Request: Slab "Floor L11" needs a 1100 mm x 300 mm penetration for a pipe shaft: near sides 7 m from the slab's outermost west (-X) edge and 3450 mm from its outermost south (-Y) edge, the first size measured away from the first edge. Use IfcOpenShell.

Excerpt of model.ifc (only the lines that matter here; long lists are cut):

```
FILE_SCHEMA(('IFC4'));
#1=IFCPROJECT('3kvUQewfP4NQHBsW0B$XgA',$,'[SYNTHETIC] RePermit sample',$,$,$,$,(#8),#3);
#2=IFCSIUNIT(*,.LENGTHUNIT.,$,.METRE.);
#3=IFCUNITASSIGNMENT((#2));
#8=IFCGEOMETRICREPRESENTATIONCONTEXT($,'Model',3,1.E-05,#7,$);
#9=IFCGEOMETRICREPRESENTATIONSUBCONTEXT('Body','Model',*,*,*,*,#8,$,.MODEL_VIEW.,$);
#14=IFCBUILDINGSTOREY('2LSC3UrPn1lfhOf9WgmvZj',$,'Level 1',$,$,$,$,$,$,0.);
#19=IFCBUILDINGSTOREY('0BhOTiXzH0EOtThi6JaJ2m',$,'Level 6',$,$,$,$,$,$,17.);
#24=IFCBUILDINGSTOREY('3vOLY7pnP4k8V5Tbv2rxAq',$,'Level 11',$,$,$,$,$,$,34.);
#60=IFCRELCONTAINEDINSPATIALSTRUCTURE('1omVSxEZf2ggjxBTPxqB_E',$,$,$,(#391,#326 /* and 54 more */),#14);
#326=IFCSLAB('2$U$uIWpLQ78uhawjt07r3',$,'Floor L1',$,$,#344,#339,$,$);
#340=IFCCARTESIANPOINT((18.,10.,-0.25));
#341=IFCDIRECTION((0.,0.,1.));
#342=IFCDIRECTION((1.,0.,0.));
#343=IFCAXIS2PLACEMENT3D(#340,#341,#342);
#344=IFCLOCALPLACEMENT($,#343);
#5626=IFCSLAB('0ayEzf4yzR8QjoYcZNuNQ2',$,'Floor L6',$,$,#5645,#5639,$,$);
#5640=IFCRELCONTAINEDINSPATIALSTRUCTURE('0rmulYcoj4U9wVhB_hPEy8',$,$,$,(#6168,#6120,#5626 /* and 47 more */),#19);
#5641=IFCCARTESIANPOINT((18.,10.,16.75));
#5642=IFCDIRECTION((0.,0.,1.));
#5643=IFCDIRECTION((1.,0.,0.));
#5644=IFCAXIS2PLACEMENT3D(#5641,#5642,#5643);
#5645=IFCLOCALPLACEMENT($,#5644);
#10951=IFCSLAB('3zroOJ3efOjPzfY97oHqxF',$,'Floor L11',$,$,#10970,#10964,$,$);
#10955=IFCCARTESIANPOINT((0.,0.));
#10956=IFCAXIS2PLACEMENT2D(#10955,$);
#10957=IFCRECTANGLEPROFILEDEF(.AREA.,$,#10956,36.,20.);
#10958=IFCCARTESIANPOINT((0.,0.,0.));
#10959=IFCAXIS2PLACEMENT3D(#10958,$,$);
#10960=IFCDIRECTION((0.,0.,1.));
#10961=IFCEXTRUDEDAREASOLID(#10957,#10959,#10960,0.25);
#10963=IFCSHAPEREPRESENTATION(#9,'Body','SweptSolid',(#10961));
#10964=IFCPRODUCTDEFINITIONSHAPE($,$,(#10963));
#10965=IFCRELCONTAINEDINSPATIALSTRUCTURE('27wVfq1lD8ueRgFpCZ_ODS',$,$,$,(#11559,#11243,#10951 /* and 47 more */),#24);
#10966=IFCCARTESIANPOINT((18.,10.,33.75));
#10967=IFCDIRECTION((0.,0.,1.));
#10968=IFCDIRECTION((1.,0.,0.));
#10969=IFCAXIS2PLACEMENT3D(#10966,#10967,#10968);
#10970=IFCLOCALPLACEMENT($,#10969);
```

```python
import numpy as np
import ifcopenshell
import ifcopenshell.api.feature
import ifcopenshell.api.geometry
import ifcopenshell.api.root
import ifcopenshell.geom
import ifcopenshell.util.placement
import ifcopenshell.util.representation
import ifcopenshell.util.shape
import ifcopenshell.util.unit

model = ifcopenshell.open("model.ifc")
unit_scale = ifcopenshell.util.unit.calculate_unit_scale(model)
settings = ifcopenshell.geom.settings()


def volume(element):
    """Net volume in cubic metres, openings subtracted."""
    shape = ifcopenshell.geom.create_shape(settings, element)
    return ifcopenshell.util.shape.get_volume(shape.geometry)


slab = model.by_guid("3zroOJ3efOjPzfY97oHqxF")
before = volume(slab)

# Extent in the slab's own axes, in metres. The edges named are its -X and -Y sides.
slab_shape = ifcopenshell.geom.create_shape(settings, slab)
vertices = ifcopenshell.util.shape.get_vertices(slab_shape.geometry)
x_min, y_min, bottom = vertices.min(axis=0)
top = vertices[:, 2].max()

opening = ifcopenshell.api.root.create_entity(model, ifc_class="IfcOpeningElement", name="Pipe shaft opening", predefined_type="OPENING")
context = ifcopenshell.util.representation.get_context(model, "Model", "Body", "MODEL_VIEW")
width, depth = 1.1, 0.3
outline = [(0.0, 0.0), (width, 0.0), (width, depth), (0.0, depth), (0.0, 0.0)]
# Overshoot both faces by 50 mm so the cut is clean.
shape = ifcopenshell.api.geometry.add_slab_representation(
    model, context=context, depth=top - bottom + 0.1, polyline=outline
)
ifcopenshell.api.geometry.assign_representation(model, product=opening, representation=shape)

matrix = ifcopenshell.util.placement.get_local_placement(slab.ObjectPlacement)
matrix[:, 3] = matrix @ np.append(np.array([x_min + 7, y_min + 3.45, bottom - 0.05]) / unit_scale, 1.0)
ifcopenshell.api.geometry.edit_object_placement(model, product=opening, matrix=matrix, is_si=False)
ifcopenshell.api.feature.add_feature(model, feature=opening, element=slab)

after = volume(slab)

print(f"slab volume {before:.3f} -> {after:.3f} m3")

model.write("model_v2.ifc")
```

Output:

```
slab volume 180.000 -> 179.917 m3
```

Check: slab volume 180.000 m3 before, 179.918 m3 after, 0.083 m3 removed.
